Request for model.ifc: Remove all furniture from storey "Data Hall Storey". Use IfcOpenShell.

First a look at what the model holds.

```python
import ifcopenshell
import ifcopenshell.util.element

model = ifcopenshell.open("model.ifc")
print(model.schema)
storey = next(s for s in model.by_type("IfcBuildingStorey") if s.Name == "Data Hall Storey")
furniture = [e for e in ifcopenshell.util.element.get_decomposition(storey) if e.is_a("IfcFurnishingElement")]
seen = {}
for e in furniture:
    element_type = ifcopenshell.util.element.get_type(e)
    name = element_type.Name if element_type not in (None, e) else None
    seen[name] = seen.get(name, 0) + 1
for name, count in sorted(seen.items(), key=str):
    print(count, "x", name)
```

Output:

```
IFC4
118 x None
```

```python
import ifcopenshell
import ifcopenshell.api.root
import ifcopenshell.util.element

model = ifcopenshell.open("model.ifc")

storey = next(s for s in model.by_type("IfcBuildingStorey") if s.Name == "Data Hall Storey")
furniture = [e for e in ifcopenshell.util.element.get_decomposition(storey) if e.is_a("IfcFurnishingElement")]

for e in furniture:
    ifcopenshell.api.root.remove_product(model, product=e)
print(len(furniture), "removed")

model.write("model_updated.ifc")
```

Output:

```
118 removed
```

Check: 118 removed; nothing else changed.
